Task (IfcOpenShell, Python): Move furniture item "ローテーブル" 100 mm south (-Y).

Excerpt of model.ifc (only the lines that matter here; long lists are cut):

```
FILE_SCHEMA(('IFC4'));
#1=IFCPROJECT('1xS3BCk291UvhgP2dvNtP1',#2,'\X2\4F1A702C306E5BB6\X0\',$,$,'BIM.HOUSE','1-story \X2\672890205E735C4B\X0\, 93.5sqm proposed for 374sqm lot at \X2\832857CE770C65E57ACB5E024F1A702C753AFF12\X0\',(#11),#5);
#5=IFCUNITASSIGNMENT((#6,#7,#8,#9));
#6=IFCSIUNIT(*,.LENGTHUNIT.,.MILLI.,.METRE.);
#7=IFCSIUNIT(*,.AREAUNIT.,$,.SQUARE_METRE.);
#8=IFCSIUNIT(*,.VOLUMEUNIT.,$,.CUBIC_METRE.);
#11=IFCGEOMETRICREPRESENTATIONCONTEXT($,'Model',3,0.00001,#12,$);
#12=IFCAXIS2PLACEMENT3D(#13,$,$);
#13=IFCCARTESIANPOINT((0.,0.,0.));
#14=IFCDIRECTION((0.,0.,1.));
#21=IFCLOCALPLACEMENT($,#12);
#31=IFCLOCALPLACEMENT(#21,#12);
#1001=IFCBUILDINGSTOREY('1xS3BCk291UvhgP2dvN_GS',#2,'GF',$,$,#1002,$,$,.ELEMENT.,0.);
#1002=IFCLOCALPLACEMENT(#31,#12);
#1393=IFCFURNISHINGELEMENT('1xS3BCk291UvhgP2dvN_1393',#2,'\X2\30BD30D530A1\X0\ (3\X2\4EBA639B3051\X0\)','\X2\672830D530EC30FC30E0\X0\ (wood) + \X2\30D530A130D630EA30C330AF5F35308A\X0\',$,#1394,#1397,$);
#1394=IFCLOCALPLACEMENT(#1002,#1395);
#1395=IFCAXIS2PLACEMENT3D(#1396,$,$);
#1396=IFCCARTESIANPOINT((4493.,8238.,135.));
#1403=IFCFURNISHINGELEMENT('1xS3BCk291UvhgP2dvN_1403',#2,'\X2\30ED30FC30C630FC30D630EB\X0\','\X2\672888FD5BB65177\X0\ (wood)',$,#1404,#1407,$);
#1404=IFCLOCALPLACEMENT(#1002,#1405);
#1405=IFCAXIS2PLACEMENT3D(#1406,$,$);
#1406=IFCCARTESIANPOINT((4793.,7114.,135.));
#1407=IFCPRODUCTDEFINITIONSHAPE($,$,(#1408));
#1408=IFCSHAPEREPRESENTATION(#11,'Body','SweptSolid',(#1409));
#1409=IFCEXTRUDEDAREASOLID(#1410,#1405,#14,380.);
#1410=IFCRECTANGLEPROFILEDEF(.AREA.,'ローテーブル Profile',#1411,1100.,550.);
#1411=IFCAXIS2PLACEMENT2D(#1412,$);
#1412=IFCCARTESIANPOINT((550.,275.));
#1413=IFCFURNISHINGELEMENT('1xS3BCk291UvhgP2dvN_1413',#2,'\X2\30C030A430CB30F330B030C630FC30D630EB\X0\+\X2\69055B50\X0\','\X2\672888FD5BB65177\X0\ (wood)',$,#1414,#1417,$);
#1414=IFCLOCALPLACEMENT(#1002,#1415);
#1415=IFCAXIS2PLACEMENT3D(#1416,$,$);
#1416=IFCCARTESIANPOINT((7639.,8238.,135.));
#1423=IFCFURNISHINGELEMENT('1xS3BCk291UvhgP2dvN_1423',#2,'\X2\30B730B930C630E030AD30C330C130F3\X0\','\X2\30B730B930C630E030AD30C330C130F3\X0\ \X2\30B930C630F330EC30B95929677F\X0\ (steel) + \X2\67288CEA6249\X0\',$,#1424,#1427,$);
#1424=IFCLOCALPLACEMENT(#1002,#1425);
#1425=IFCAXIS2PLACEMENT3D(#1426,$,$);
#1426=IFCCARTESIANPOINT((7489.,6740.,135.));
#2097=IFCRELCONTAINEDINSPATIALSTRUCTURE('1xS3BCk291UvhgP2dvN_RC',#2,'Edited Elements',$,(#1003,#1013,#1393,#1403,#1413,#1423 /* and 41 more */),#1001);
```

```python
import ifcopenshell
import ifcopenshell.api.geometry
import ifcopenshell.util.placement

model = ifcopenshell.open("model.ifc")

item = model.by_id(1403)
matrix = ifcopenshell.util.placement.get_local_placement(item.ObjectPlacement)
matrix[1, 3] -= 100.0
ifcopenshell.api.geometry.edit_object_placement(model, product=item, matrix=matrix, is_si=False)

print(ifcopenshell.util.placement.get_local_placement(item.ObjectPlacement).round(3) + 0.0)

model.write("model-out.ifc")
```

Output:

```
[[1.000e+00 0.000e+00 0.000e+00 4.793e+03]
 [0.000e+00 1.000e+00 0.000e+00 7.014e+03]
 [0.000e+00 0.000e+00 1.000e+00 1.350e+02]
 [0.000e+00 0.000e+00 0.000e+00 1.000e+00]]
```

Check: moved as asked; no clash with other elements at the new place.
